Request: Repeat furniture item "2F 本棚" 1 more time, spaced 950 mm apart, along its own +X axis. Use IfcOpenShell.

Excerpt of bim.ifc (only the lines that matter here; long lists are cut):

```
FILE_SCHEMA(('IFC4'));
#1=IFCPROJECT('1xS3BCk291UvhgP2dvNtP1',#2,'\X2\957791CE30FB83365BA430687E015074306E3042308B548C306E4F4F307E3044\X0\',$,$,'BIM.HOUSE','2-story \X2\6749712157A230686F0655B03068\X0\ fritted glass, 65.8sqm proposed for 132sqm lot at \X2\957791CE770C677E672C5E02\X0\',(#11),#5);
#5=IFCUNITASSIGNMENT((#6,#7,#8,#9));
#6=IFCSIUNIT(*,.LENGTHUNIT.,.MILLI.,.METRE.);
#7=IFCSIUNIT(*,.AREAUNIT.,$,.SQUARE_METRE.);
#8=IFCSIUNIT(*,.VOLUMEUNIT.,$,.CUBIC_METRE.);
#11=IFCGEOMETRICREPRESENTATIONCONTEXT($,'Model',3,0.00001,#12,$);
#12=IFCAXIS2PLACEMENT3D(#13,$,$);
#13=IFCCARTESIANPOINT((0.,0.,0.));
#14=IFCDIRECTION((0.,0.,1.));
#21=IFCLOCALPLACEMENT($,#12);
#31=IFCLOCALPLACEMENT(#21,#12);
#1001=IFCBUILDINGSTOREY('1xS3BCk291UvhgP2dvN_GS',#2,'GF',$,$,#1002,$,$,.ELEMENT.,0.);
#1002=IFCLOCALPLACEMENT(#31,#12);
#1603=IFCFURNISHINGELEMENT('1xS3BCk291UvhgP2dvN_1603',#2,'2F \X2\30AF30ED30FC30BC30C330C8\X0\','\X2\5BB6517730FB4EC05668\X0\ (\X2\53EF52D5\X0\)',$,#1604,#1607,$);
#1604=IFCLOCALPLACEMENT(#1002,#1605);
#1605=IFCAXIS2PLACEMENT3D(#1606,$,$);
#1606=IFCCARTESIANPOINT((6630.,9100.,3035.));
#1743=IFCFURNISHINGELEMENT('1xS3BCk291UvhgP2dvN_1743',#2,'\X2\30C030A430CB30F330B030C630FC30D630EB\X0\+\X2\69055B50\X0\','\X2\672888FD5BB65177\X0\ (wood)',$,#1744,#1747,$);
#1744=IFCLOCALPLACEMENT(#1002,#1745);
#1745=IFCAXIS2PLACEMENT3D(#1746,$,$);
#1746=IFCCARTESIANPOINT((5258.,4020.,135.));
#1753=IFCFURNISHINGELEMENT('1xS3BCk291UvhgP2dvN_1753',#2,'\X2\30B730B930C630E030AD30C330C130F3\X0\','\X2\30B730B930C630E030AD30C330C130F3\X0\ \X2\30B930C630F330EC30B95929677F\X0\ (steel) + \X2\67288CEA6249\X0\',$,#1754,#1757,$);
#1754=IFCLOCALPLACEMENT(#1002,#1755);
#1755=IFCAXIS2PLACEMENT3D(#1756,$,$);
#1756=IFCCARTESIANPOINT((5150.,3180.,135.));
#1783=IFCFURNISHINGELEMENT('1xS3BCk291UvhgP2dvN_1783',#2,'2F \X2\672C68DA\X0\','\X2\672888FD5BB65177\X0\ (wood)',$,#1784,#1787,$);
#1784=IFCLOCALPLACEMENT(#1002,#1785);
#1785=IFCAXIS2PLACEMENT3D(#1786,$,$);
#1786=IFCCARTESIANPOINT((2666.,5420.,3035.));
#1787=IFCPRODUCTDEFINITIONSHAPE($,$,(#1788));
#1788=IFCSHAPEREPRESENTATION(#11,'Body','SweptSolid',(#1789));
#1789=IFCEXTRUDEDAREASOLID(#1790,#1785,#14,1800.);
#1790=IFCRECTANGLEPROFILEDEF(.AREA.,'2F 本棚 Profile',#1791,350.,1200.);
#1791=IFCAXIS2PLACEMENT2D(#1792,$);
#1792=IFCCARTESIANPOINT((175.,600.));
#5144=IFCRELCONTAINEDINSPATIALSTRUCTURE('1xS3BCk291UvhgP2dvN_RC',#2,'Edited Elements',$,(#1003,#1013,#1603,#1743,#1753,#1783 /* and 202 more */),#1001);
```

```python
import ifcopenshell
import ifcopenshell.api.geometry
import ifcopenshell.api.root
import ifcopenshell.util.element
import ifcopenshell.util.placement

model = ifcopenshell.open("bim.ifc")


def reuse_history(source, copy):
    """copy_class also copies each property set's owner history, people and application; keep the originals."""
    for rel in copy.IsDefinedBy:
        if rel.is_a("IfcRelDefinesByProperties") and (history := rel.RelatingPropertyDefinition.OwnerHistory):
            rel.RelatingPropertyDefinition.OwnerHistory = source.OwnerHistory
            ifcopenshell.util.element.remove_deep2(model, history)


source = model.by_guid("1xS3BCk291UvhgP2dvN_1783")
base = ifcopenshell.util.placement.get_local_placement(source.ObjectPlacement)
step = base[:3, 0] * 950.0

for i in range(1, 2):
    copy = ifcopenshell.api.root.copy_class(model, product=source)
    copy.Representation = ifcopenshell.util.element.copy_deep(
        model, source.Representation, exclude=["IfcGeometricRepresentationContext", "IfcRepresentationMap"]
    )
    reuse_history(source, copy)
    matrix = base.copy()
    matrix[:3, 3] += i * step
    print("added at", matrix[:3, 3].round(3) + 0.0)
    ifcopenshell.api.geometry.edit_object_placement(model, product=copy, matrix=matrix, is_si=False)

model.write("bim-out.ifc")
```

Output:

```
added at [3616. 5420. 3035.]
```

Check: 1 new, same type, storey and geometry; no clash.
